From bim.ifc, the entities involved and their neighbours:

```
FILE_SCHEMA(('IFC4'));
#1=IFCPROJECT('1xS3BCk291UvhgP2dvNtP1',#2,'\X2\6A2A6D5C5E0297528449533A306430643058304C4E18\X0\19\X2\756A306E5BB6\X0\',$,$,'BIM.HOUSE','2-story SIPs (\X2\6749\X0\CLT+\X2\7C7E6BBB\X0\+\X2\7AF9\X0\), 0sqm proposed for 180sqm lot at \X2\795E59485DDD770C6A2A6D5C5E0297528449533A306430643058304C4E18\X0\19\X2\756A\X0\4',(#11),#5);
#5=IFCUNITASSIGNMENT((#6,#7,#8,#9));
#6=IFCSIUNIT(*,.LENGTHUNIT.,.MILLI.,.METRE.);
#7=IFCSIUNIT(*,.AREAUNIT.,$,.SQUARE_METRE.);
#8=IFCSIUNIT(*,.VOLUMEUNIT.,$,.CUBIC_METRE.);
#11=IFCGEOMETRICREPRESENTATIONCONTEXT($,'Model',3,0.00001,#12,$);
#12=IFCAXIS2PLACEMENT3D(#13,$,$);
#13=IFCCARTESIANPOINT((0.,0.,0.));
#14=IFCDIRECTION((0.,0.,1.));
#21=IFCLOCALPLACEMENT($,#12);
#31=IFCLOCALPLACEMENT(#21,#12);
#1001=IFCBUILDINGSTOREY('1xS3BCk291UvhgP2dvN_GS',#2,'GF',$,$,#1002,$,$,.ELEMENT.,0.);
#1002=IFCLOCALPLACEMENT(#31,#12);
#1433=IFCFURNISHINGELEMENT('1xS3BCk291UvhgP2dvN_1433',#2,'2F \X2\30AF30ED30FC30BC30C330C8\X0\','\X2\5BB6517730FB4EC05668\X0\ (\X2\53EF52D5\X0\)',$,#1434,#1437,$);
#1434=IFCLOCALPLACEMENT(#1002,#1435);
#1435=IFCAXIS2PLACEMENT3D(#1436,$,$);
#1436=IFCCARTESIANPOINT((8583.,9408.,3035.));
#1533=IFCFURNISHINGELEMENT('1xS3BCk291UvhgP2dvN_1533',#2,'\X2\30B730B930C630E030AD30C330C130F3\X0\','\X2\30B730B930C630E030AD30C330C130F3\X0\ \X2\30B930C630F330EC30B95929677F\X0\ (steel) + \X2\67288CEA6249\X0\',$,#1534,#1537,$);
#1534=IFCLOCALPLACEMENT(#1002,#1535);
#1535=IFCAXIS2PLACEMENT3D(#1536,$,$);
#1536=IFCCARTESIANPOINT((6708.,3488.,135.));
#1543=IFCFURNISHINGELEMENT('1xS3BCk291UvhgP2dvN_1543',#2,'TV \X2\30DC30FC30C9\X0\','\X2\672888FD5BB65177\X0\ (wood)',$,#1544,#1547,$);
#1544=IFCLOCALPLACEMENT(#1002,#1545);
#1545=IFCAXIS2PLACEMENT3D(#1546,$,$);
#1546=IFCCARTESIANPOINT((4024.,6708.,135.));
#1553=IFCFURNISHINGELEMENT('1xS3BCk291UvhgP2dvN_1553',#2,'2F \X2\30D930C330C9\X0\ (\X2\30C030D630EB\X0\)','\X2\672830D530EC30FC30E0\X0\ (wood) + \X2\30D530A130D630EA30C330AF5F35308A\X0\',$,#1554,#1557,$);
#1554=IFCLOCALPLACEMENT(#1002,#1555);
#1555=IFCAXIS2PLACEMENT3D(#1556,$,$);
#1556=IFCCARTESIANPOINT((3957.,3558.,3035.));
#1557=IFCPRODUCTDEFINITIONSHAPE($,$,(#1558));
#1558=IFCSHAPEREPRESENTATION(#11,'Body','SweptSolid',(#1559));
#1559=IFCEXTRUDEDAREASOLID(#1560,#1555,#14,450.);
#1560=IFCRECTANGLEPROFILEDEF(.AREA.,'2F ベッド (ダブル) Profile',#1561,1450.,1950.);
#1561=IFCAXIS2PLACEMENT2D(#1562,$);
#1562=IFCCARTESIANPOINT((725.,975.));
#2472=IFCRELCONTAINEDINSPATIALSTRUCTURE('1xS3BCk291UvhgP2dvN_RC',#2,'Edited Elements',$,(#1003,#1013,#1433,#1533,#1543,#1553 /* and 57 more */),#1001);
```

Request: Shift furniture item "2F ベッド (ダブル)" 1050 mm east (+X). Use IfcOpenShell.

```python
import ifcopenshell
import ifcopenshell.api.geometry
import ifcopenshell.util.placement

model = ifcopenshell.open("bim.ifc")

item = model.by_guid("1xS3BCk291UvhgP2dvN_1553")
matrix = ifcopenshell.util.placement.get_local_placement(item.ObjectPlacement)
matrix[0, 3] += 1050.0
ifcopenshell.api.geometry.edit_object_placement(model, product=item, matrix=matrix, is_si=False)

print(ifcopenshell.util.placement.get_local_placement(item.ObjectPlacement).round(3) + 0.0)

model.write("bim_rev.ifc")
```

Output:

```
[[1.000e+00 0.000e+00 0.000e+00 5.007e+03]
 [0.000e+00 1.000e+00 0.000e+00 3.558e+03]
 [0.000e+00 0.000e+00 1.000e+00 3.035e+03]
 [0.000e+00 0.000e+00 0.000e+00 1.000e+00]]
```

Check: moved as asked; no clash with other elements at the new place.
